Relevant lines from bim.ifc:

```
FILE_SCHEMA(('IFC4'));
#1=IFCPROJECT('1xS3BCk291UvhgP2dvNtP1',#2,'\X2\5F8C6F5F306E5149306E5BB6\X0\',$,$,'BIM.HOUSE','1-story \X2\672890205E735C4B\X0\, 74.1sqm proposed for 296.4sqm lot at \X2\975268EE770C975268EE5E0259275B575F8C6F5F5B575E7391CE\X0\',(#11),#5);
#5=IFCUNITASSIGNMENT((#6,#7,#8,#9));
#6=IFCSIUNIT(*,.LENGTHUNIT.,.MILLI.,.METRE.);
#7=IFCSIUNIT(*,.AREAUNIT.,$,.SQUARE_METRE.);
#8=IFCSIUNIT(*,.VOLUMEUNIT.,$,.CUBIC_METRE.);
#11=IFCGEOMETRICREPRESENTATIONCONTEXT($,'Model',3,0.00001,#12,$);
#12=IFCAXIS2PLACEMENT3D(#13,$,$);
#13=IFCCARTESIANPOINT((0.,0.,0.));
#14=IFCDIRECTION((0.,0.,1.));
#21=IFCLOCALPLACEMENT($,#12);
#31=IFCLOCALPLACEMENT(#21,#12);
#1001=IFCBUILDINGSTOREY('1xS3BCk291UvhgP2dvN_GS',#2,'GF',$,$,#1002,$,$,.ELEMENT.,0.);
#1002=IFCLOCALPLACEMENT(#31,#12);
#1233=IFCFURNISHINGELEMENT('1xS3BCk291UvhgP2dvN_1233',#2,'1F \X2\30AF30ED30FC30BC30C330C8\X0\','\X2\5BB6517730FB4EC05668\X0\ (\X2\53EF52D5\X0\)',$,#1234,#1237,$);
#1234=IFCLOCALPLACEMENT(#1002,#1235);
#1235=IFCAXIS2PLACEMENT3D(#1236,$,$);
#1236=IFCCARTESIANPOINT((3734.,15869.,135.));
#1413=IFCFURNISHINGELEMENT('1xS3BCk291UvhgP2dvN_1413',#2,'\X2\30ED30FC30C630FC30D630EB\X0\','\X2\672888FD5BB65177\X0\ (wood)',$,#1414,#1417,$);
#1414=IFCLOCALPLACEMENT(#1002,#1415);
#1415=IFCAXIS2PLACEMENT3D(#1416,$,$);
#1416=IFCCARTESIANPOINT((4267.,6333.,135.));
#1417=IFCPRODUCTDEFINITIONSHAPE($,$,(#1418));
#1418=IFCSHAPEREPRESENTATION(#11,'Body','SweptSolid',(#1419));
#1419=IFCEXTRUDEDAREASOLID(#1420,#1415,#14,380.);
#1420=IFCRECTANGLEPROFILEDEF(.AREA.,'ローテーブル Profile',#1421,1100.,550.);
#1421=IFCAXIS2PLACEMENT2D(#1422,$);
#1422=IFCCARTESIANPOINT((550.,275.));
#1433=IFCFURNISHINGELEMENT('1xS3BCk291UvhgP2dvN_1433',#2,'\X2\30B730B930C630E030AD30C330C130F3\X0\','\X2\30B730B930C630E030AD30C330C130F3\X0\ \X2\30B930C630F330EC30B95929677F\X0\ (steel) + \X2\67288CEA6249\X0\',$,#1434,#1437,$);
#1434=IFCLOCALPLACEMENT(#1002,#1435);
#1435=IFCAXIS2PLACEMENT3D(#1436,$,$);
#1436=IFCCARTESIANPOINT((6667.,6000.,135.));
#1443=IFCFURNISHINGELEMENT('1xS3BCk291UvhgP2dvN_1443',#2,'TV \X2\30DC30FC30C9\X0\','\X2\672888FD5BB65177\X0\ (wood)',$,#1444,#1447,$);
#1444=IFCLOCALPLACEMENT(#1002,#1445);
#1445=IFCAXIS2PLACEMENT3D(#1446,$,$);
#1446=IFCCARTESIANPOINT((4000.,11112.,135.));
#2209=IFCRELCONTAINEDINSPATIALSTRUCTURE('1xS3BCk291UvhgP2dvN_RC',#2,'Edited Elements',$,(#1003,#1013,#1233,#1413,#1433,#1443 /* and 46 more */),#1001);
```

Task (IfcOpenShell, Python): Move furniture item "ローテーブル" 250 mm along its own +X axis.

```python
import ifcopenshell
import ifcopenshell.api.geometry
import ifcopenshell.util.placement
import ifcopenshell.util.unit

model = ifcopenshell.open("bim.ifc")
unit_scale = ifcopenshell.util.unit.calculate_unit_scale(model)

item = model.by_guid("1xS3BCk291UvhgP2dvN_1413")
matrix = ifcopenshell.util.placement.get_local_placement(item.ObjectPlacement)
matrix[:3, 3] += matrix[:3, 0] * 0.25 / unit_scale
ifcopenshell.api.geometry.edit_object_placement(model, product=item, matrix=matrix, is_si=False)

print(ifcopenshell.util.placement.get_local_placement(item.ObjectPlacement).round(3) + 0.0)

model.write("bim_rev.ifc")
```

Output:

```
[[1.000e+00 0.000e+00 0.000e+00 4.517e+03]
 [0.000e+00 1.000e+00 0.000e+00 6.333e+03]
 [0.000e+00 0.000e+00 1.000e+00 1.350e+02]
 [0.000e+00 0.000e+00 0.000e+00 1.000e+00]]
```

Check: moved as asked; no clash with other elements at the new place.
